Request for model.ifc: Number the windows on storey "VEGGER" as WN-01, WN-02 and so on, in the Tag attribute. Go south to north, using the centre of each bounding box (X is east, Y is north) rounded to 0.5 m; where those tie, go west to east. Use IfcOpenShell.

First a look at what the model holds.

```python
import ifcopenshell
import ifcopenshell.util.element
import ifcopenshell.util.placement

model = ifcopenshell.open("model.ifc")
print(model.schema)
storey = next(s for s in model.by_type("IfcBuildingStorey") if s.Name == "VEGGER")
windows = [e for e in ifcopenshell.util.element.get_decomposition(storey) if e.is_a("IfcWindow")]
for e in sorted(windows, key=lambda e: e.id()):
    origin = ifcopenshell.util.placement.get_local_placement(e.ObjectPlacement)[:3, 3]
    print(e.id(), e.Tag, e.Name, origin.round(2) + 0.0, sep=" | ")
```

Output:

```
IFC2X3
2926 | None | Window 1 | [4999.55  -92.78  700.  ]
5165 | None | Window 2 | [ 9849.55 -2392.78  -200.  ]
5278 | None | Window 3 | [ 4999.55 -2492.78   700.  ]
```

```python
import ifcopenshell
import ifcopenshell.geom
import ifcopenshell.util.element
import ifcopenshell.util.shape

model = ifcopenshell.open("model.ifc")
settings = ifcopenshell.geom.settings()
settings.set("use-world-coords", True)


def centre(element):
    shape = ifcopenshell.geom.create_shape(settings, element)
    return ifcopenshell.util.shape.get_bbox_centroid(shape.geometry)


storey = next(s for s in model.by_type("IfcBuildingStorey") if s.Name == "VEGGER")
windows = [e for e in ifcopenshell.util.element.get_decomposition(storey) if e.is_a("IfcWindow")]

# Insertion points can sit at a corner or the storey origin, so sort by the geometry (in metres).
centres = {e: centre(e) for e in windows}
windows.sort(key=lambda e: (round(centres[e][1] / 0.5), centres[e][0]))

for i, e in enumerate(windows, start=1):
    number = f"WN-{i:02d}"
    e.Tag = number
    print(e.id(), number)

model.write("model_edited.ifc")
```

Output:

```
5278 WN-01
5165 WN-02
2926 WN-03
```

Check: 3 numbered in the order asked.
